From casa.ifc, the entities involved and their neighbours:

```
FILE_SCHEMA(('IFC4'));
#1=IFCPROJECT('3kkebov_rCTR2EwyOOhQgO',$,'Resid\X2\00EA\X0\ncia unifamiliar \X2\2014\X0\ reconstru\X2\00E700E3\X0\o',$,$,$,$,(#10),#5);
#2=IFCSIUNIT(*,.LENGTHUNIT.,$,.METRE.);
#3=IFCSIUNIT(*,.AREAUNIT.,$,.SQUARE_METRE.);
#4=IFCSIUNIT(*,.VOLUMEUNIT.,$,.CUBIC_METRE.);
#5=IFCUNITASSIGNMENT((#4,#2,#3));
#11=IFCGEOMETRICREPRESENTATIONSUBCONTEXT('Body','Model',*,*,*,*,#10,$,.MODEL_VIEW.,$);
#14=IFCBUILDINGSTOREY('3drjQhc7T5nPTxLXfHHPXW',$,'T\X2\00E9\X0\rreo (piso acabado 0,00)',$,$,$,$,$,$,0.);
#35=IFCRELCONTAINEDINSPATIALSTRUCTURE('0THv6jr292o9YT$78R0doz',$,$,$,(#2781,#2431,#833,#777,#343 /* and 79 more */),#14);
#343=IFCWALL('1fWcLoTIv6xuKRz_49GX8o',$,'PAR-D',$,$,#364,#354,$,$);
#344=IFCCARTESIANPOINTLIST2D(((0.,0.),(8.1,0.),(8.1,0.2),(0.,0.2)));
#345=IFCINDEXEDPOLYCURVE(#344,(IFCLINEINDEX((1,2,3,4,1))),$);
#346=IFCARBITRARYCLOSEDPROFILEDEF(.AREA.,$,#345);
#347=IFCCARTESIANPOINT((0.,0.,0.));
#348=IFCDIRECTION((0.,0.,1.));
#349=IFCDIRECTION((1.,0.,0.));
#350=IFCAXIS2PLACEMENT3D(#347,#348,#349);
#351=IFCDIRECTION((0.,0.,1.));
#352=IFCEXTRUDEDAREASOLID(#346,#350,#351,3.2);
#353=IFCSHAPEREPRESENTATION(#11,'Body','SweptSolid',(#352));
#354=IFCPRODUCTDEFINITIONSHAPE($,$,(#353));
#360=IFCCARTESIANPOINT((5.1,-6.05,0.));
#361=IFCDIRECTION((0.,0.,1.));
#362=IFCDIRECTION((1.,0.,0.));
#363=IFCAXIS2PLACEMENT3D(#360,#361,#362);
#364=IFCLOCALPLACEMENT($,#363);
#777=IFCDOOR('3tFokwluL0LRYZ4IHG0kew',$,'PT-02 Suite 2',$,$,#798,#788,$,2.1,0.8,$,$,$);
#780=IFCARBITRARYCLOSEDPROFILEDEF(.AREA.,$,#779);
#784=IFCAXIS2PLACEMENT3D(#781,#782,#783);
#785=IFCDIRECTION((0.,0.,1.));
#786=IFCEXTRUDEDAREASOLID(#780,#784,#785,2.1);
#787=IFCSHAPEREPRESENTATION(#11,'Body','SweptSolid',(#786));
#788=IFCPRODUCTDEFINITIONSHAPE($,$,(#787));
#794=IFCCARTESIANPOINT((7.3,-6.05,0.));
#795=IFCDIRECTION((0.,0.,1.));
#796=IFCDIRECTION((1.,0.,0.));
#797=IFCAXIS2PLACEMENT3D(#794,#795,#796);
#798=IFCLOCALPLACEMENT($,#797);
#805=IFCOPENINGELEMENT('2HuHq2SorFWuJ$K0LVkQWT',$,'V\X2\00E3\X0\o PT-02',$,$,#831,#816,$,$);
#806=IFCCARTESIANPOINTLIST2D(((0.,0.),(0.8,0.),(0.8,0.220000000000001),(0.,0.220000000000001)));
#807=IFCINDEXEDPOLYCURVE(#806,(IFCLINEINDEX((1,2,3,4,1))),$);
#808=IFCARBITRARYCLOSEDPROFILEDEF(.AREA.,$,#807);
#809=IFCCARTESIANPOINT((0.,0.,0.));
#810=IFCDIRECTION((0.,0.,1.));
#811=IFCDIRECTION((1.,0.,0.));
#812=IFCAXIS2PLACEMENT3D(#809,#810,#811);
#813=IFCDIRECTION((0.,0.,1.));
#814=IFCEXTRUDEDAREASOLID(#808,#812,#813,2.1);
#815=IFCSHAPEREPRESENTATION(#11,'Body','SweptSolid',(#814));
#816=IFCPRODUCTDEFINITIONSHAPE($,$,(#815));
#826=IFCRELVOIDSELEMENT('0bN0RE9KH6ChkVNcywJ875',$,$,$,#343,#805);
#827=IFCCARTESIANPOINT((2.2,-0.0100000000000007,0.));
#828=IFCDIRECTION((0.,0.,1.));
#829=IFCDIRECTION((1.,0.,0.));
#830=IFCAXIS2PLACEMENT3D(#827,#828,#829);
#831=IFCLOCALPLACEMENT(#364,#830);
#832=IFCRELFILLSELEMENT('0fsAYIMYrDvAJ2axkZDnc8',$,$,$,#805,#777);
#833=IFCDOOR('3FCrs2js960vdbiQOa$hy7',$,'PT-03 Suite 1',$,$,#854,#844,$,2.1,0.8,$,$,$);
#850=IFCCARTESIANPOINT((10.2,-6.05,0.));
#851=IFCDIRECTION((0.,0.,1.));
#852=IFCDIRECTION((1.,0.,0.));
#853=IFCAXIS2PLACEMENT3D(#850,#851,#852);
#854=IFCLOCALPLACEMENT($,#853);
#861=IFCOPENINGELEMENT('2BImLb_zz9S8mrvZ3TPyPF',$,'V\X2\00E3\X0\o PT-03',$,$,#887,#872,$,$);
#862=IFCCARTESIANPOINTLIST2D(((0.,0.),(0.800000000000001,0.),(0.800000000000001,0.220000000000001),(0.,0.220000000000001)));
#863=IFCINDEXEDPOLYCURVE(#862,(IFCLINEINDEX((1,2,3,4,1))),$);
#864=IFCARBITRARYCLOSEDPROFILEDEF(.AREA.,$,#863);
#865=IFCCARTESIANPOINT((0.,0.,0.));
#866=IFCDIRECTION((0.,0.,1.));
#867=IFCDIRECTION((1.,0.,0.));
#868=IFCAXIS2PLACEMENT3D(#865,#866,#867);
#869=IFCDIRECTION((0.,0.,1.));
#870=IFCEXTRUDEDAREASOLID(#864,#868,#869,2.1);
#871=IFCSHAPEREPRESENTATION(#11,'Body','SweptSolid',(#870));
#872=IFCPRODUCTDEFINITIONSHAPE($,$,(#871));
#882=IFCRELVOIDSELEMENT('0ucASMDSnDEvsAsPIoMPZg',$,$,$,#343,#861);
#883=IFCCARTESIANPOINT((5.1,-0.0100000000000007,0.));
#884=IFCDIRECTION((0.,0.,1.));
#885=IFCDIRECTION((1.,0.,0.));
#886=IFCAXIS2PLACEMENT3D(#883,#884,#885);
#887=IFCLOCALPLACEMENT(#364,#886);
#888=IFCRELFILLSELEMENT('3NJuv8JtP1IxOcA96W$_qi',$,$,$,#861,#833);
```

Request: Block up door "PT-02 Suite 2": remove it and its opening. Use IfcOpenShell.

```python
import ifcopenshell
import ifcopenshell.api.feature
import ifcopenshell.api.root
import ifcopenshell.geom
import ifcopenshell.util.shape

model = ifcopenshell.open("casa.ifc")
settings = ifcopenshell.geom.settings()


def volume(element):
    """Net volume in cubic metres, openings subtracted."""
    shape = ifcopenshell.geom.create_shape(settings, element)
    return ifcopenshell.util.shape.get_volume(shape.geometry)


door = model.by_id(777)
opening = door.FillsVoids[0].RelatingOpeningElement
wall = opening.VoidsElements[0].RelatingBuildingElement
before = volume(wall)

ifcopenshell.api.root.remove_product(model, product=door)
ifcopenshell.api.feature.remove_feature(model, feature=opening)

after = volume(wall)

print(f"wall volume {before:.3f} -> {after:.3f} m3")

model.write("casa_edited.ifc")
```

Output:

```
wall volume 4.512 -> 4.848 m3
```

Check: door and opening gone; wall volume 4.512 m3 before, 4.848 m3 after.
